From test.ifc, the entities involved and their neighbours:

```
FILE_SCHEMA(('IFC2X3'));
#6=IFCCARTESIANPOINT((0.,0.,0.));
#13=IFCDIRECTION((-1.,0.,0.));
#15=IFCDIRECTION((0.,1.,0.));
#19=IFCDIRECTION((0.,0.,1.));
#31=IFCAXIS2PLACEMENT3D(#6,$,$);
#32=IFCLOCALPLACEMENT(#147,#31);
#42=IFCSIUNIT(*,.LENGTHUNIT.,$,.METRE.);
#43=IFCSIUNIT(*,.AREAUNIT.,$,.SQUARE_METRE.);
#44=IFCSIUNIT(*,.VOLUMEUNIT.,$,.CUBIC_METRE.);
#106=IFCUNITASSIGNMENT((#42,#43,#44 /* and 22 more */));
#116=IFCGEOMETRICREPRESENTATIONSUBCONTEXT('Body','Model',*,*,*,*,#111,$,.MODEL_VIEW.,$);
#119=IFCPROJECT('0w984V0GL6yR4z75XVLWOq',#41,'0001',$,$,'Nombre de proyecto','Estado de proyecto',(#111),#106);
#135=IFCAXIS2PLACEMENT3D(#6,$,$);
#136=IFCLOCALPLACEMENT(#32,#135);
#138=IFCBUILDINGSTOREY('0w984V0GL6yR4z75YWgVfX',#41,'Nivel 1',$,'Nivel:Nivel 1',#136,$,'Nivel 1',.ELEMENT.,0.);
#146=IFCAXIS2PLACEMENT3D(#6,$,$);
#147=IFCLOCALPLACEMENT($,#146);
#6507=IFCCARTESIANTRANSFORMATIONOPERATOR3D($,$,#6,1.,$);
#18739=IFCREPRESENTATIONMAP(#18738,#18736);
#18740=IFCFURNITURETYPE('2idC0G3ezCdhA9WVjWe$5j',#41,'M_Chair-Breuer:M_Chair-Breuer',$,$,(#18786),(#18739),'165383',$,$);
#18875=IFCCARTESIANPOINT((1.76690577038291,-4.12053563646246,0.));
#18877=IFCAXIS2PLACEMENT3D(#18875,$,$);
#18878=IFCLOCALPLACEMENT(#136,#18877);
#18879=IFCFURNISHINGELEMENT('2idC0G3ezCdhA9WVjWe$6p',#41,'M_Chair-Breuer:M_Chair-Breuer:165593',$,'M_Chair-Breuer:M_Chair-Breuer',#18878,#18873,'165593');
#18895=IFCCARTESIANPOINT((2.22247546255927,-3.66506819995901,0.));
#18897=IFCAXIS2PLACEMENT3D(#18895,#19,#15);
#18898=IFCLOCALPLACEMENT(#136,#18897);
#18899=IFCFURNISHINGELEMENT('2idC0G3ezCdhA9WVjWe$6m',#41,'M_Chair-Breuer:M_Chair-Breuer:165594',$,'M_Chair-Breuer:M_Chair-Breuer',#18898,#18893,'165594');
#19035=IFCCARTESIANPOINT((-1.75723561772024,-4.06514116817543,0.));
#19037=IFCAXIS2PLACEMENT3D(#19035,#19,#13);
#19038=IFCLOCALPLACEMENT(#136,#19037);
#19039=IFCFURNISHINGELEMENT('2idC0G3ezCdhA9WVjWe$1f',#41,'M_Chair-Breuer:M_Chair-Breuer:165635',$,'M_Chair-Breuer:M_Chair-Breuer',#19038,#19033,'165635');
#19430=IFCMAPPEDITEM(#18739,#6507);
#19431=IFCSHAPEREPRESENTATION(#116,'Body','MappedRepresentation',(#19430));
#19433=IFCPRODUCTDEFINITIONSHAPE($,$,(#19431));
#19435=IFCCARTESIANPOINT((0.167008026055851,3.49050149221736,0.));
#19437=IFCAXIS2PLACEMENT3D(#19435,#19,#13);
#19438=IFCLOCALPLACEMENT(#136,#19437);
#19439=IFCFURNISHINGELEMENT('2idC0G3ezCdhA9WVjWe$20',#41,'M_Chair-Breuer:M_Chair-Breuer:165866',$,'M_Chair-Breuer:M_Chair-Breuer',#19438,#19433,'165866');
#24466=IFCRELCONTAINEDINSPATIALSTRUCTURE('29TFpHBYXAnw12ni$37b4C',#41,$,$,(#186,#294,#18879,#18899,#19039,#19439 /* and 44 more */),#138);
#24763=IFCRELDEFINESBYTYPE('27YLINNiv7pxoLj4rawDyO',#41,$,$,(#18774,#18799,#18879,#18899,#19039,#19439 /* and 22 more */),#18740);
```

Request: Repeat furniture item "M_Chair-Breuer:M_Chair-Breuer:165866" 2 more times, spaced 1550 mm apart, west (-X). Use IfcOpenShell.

```python
import numpy as np
import ifcopenshell
import ifcopenshell.api.geometry
import ifcopenshell.api.root
import ifcopenshell.util.element
import ifcopenshell.util.placement
import ifcopenshell.util.unit

model = ifcopenshell.open("test.ifc")
unit_scale = ifcopenshell.util.unit.calculate_unit_scale(model)


def reuse_history(source, copy):
    """copy_class also copies each property set's owner history, people and application; keep the originals."""
    for rel in copy.IsDefinedBy:
        if rel.is_a("IfcRelDefinesByProperties") and (history := rel.RelatingPropertyDefinition.OwnerHistory):
            rel.RelatingPropertyDefinition.OwnerHistory = source.OwnerHistory
            ifcopenshell.util.element.remove_deep2(model, history)


source = model.by_id(19439)
base = ifcopenshell.util.placement.get_local_placement(source.ObjectPlacement)
step = np.array([-1.0, 0.0, 0.0]) * 1.55 / unit_scale

for i in range(1, 3):
    copy = ifcopenshell.api.root.copy_class(model, product=source)
    copy.Representation = ifcopenshell.util.element.copy_deep(
        model, source.Representation, exclude=["IfcGeometricRepresentationContext", "IfcRepresentationMap"]
    )
    copy.Name = "M_Chair-Breuer:M_Chair-Breuer"
    copy.Tag = None
    reuse_history(source, copy)
    matrix = base.copy()
    matrix[:3, 3] += i * step
    print("added at", matrix[:3, 3].round(3) + 0.0)
    ifcopenshell.api.geometry.edit_object_placement(model, product=copy, matrix=matrix, is_si=False)

model.write("test_updated.ifc")
```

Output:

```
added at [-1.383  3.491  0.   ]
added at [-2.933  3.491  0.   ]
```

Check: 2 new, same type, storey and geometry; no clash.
